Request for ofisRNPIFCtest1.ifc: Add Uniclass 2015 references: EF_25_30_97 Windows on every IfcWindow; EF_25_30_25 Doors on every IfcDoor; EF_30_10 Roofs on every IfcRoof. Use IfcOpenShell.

First a look at what the model holds.

```python
import ifcopenshell

model = ifcopenshell.open("ofisRNPIFCtest1.ifc")
print(model.schema)
print("classifications:", [c.Name for c in model.by_type("IfcClassification")])
for ifc_class in ("IfcDoor", "IfcRoof", "IfcStair", "IfcWall", "IfcWindow"):
    print(ifc_class, len(model.by_type(ifc_class)))
```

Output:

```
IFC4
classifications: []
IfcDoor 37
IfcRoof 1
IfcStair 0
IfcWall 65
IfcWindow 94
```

```python
import ifcopenshell
import ifcopenshell.api.classification

model = ifcopenshell.open("ofisRNPIFCtest1.ifc")

system = ifcopenshell.api.classification.add_classification(model, classification="Uniclass 2015")

codes = {
    "IfcWindow": ("EF_25_30_97", "Windows"),
    "IfcDoor": ("EF_25_30_25", "Doors"),
    "IfcRoof": ("EF_30_10", "Roofs"),
}
for ifc_class, (code, name) in codes.items():
    products = model.by_type(ifc_class)
    ifcopenshell.api.classification.add_reference(
        model, products=products, classification=system, identification=code, name=name
    )
    print(code, len(products))

model.write("ofisRNPIFCtest1_rev.ifc")
```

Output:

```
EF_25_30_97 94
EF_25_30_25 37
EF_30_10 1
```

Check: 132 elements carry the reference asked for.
